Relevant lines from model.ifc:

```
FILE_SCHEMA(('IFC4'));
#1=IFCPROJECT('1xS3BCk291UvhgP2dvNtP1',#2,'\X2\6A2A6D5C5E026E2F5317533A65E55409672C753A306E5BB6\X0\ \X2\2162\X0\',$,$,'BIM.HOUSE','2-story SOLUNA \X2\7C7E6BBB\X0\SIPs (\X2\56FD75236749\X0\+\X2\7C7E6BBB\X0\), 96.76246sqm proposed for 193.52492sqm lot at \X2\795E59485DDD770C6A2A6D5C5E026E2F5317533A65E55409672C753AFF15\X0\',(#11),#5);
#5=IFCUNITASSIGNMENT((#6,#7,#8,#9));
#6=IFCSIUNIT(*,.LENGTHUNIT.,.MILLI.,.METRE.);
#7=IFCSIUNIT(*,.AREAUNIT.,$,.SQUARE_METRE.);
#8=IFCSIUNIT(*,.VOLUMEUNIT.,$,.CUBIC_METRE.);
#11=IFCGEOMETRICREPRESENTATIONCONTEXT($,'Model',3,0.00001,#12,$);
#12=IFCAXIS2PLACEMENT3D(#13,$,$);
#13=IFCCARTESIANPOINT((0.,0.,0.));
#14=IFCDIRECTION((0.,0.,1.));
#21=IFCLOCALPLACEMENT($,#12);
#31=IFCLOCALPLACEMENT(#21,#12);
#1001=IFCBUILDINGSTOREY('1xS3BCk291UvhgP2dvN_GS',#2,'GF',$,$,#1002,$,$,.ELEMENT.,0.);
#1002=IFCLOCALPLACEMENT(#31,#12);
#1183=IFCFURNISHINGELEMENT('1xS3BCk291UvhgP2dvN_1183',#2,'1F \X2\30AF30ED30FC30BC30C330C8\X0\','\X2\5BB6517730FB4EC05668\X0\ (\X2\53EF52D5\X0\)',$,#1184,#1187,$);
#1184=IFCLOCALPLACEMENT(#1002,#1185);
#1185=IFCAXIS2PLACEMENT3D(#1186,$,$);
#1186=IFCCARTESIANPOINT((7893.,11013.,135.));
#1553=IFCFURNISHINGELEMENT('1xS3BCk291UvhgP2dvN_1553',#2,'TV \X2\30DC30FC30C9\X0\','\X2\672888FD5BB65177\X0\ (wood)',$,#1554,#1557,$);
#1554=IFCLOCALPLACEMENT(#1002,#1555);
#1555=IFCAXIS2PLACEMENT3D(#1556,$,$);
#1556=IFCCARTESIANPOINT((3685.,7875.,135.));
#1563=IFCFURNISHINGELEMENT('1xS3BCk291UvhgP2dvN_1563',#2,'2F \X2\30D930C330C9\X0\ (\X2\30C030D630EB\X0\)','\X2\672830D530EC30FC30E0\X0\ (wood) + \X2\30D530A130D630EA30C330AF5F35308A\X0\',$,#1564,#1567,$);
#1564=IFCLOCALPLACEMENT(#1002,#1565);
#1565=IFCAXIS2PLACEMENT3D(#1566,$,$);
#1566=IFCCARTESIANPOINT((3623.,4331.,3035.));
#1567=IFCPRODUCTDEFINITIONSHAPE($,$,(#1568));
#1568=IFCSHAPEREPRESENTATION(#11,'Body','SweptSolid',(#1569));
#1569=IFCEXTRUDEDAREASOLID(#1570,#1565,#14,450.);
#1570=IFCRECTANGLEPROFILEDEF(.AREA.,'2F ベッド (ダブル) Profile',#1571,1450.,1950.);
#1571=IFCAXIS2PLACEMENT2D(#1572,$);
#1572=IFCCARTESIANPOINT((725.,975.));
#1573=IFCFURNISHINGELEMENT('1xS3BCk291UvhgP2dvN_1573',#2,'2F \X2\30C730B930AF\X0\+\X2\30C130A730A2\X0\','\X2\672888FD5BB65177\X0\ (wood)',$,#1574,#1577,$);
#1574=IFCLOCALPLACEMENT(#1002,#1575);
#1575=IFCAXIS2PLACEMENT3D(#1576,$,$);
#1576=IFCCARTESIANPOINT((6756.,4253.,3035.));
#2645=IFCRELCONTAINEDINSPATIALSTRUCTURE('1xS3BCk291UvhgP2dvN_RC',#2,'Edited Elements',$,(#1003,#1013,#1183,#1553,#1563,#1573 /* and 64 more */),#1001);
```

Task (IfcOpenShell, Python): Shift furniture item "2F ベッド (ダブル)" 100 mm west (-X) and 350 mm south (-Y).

```python
import ifcopenshell
import ifcopenshell.api.geometry
import ifcopenshell.util.placement
import ifcopenshell.util.unit

model = ifcopenshell.open("model.ifc")
unit_scale = ifcopenshell.util.unit.calculate_unit_scale(model)

item = model.by_guid("1xS3BCk291UvhgP2dvN_1563")
matrix = ifcopenshell.util.placement.get_local_placement(item.ObjectPlacement)
matrix[0, 3] -= 0.1 / unit_scale
matrix[1, 3] -= 0.35 / unit_scale
ifcopenshell.api.geometry.edit_object_placement(model, product=item, matrix=matrix, is_si=False)

print(ifcopenshell.util.placement.get_local_placement(item.ObjectPlacement).round(3) + 0.0)

model.write("model_updated.ifc")
```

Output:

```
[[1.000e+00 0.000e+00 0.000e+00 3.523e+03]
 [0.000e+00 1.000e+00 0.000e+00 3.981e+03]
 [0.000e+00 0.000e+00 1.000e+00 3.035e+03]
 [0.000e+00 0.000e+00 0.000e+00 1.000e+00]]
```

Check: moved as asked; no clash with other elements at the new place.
